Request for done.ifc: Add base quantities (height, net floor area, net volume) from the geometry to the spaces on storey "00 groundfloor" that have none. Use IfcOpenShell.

First a look at what the model holds.

```python
import ifcopenshell
import ifcopenshell.util.element
import ifcopenshell.util.unit

model = ifcopenshell.open("done.ifc")
print(model.schema)
for unit_type in ("LENGTHUNIT", "AREAUNIT", "VOLUMEUNIT"):
    print(unit_type, ifcopenshell.util.unit.calculate_unit_scale(model, unit_type))
storey = next(s for s in model.by_type("IfcBuildingStorey") if s.Name == "00 groundfloor")
spaces = [e for e in ifcopenshell.util.element.get_decomposition(storey) if e.is_a("IfcSpace")]
for e in sorted(spaces, key=lambda e: e.id()):
    print(e.id(), e.is_a(), e.Name, list(ifcopenshell.util.element.get_psets(e, qtos_only=True)), sep=" | ")
```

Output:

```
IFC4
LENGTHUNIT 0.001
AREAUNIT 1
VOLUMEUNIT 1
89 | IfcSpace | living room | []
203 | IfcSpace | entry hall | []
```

```python
import ifcopenshell
import ifcopenshell.api.pset
import ifcopenshell.geom
import ifcopenshell.util.element
import ifcopenshell.util.shape
import ifcopenshell.util.unit

model = ifcopenshell.open("done.ifc")
unit_scale = ifcopenshell.util.unit.calculate_unit_scale(model)
area_scale = ifcopenshell.util.unit.calculate_unit_scale(model, "AREAUNIT")
volume_scale = ifcopenshell.util.unit.calculate_unit_scale(model, "VOLUMEUNIT")
settings = ifcopenshell.geom.settings()

storey = next(s for s in model.by_type("IfcBuildingStorey") if s.Name == "00 groundfloor")
spaces = [e for e in ifcopenshell.util.element.get_decomposition(storey) if e.is_a("IfcSpace")]

for e in sorted(spaces, key=lambda e: e.id()):
    if ifcopenshell.util.element.get_psets(e, qtos_only=True, should_inherit=False):
        continue
    # Geometry comes back in metres, in the element's own axes.
    shape = ifcopenshell.geom.create_shape(settings, e)
    values = {
        "Height": ifcopenshell.util.shape.get_z(shape.geometry) / unit_scale,
        "NetFloorArea": ifcopenshell.util.shape.get_footprint_area(shape.geometry) / area_scale,
        "NetVolume": ifcopenshell.util.shape.get_volume(shape.geometry) / volume_scale,
    }
    qto = ifcopenshell.api.pset.add_qto(model, product=e, name="Qto_SpaceBaseQuantities")
    ifcopenshell.api.pset.edit_qto(model, qto=qto, properties=values)
    print(e.id(), {k: round(v, 3) for k, v in values.items()})

model.write("done-out.ifc")
```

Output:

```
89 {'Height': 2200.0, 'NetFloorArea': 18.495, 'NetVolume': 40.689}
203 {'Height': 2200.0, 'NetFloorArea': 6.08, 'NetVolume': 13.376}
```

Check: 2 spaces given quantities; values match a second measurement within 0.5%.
